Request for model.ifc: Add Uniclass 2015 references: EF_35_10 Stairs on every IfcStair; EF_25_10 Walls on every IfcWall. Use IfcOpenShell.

First a look at what the model holds.

```python
import ifcopenshell

model = ifcopenshell.open("model.ifc")
print(model.schema)
print("classifications:", [c.Name for c in model.by_type("IfcClassification")])
for ifc_class in ("IfcDoor", "IfcRoof", "IfcStair", "IfcWall", "IfcWindow"):
    print(ifc_class, len(model.by_type(ifc_class)))
```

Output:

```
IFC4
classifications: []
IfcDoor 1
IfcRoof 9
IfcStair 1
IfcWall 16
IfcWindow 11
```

```python
import ifcopenshell
import ifcopenshell.api.classification

model = ifcopenshell.open("model.ifc")

system = ifcopenshell.api.classification.add_classification(model, classification="Uniclass 2015")

codes = {
    "IfcStair": ("EF_35_10", "Stairs"),
    "IfcWall": ("EF_25_10", "Walls"),
}
for ifc_class, (code, name) in codes.items():
    products = model.by_type(ifc_class)
    ifcopenshell.api.classification.add_reference(
        model, products=products, classification=system, identification=code, name=name
    )
    print(code, len(products))

model.write("model_updated.ifc")
```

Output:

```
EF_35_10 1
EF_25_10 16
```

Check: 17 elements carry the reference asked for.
